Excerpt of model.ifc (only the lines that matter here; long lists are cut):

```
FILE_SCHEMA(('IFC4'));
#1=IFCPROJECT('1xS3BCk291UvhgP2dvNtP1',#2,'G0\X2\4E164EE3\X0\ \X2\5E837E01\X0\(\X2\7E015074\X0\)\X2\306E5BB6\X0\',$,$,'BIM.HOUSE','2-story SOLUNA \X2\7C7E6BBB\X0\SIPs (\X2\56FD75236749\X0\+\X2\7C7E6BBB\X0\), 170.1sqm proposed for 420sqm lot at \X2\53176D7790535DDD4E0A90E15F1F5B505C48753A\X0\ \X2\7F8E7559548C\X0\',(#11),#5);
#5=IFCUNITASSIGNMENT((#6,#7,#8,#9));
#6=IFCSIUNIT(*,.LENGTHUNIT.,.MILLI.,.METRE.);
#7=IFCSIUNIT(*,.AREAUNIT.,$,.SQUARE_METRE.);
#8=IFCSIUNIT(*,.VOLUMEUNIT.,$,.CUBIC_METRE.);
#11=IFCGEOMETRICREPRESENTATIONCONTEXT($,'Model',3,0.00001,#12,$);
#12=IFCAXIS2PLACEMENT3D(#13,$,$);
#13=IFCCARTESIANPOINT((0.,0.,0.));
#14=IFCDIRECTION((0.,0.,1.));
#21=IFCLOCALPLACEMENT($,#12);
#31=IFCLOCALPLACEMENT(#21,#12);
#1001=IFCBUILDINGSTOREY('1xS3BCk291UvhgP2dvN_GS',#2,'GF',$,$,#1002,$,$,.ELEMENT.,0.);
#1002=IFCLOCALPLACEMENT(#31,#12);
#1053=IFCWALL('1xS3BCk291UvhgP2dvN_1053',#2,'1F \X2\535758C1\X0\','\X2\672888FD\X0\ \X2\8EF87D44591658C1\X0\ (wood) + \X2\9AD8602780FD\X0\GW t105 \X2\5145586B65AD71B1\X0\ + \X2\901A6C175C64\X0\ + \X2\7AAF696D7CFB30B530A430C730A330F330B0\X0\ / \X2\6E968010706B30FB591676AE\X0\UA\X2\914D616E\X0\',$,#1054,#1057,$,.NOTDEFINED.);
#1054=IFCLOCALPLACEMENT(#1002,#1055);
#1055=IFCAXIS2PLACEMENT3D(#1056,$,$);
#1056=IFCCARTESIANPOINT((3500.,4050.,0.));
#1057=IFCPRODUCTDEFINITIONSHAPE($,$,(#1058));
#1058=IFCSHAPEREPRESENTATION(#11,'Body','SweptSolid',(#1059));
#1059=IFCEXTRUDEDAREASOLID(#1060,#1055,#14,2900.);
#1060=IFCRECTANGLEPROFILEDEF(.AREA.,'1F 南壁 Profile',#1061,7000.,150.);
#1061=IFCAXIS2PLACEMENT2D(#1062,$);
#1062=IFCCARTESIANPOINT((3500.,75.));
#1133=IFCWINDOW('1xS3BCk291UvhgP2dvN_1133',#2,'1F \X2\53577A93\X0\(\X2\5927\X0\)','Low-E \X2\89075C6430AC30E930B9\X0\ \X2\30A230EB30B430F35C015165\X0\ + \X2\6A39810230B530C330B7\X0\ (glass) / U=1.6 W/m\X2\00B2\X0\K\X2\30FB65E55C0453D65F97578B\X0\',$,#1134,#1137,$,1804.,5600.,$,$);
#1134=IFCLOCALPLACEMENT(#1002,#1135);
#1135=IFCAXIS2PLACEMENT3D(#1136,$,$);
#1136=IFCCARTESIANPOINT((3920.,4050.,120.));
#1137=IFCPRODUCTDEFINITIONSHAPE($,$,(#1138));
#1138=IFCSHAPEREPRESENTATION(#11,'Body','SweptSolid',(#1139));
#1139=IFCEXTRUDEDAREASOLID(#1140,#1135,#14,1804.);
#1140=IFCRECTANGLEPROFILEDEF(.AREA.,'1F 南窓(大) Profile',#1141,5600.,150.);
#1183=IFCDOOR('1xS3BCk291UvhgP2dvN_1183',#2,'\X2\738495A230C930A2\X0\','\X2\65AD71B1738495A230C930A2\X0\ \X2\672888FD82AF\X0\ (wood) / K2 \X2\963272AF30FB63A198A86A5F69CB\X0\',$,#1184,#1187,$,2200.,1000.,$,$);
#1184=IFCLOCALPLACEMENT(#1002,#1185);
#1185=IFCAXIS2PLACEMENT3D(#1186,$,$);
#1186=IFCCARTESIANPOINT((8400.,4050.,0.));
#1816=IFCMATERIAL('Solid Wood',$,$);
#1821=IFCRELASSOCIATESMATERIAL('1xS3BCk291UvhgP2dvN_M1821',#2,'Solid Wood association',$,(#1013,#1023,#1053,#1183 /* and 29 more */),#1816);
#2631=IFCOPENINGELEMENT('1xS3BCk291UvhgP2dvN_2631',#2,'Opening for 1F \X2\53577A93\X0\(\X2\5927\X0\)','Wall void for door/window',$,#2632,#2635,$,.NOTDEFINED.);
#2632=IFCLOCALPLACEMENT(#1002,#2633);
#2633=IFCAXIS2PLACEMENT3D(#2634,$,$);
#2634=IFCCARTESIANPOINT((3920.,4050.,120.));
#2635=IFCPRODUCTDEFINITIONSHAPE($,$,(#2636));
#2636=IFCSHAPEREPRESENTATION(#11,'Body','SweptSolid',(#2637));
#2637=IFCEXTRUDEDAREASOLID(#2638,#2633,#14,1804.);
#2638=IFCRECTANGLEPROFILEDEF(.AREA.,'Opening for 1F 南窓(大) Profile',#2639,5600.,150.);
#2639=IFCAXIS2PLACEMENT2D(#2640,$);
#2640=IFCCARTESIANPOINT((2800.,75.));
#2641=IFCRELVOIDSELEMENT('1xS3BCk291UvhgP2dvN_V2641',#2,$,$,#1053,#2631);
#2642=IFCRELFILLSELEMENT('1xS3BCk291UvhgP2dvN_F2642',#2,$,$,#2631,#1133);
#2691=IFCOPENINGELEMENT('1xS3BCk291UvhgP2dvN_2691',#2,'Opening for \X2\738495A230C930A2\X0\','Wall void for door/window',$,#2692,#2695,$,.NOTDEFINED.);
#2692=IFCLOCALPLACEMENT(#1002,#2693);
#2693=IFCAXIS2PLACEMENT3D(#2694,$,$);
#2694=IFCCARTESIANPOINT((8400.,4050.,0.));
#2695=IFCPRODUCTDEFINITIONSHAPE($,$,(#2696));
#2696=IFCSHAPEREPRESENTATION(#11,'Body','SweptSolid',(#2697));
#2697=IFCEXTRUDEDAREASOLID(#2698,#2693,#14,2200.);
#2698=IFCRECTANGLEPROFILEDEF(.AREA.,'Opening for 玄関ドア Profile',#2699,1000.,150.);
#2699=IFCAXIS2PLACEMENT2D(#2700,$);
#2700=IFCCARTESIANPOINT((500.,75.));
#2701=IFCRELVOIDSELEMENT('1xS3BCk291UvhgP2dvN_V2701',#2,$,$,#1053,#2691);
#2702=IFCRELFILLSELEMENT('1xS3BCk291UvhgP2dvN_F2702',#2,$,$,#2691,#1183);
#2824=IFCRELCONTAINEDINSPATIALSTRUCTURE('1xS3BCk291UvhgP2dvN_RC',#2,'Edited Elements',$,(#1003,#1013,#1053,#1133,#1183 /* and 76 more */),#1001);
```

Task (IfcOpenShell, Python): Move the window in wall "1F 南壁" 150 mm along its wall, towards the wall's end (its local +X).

```python
import ifcopenshell
import ifcopenshell.api.geometry
import ifcopenshell.util.placement
import ifcopenshell.util.unit

model = ifcopenshell.open("model.ifc")
unit_scale = ifcopenshell.util.unit.calculate_unit_scale(model)

window = model.by_guid("1xS3BCk291UvhgP2dvN_1133")
opening = window.FillsVoids[0].RelatingOpeningElement
wall = opening.VoidsElements[0].RelatingBuildingElement

wall_matrix = ifcopenshell.util.placement.get_local_placement(wall.ObjectPlacement)
shift = wall_matrix[:3, 0] * 0.15 / unit_scale
before = ifcopenshell.util.placement.get_local_placement(window.ObjectPlacement)[:3, 3].copy()

# The window is not placed relative to its opening, so move both.
for product in (opening, window):
    matrix = ifcopenshell.util.placement.get_local_placement(product.ObjectPlacement)
    matrix[:3, 3] += shift
    ifcopenshell.api.geometry.edit_object_placement(model, product=product, matrix=matrix, is_si=False)

after = ifcopenshell.util.placement.get_local_placement(window.ObjectPlacement)[:3, 3]
print("window moved by", (after - before).round(3) + 0.0)

model.write("model_updated.ifc")
```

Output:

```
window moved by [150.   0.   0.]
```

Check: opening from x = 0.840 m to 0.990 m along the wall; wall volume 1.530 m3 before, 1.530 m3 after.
